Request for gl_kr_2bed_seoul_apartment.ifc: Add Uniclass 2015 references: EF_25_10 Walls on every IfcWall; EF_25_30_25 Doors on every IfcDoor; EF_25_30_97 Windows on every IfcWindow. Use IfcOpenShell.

First a look at what the model holds.

```python
import ifcopenshell

model = ifcopenshell.open("gl_kr_2bed_seoul_apartment.ifc")
print(model.schema)
print("classifications:", [c.Name for c in model.by_type("IfcClassification")])
for ifc_class in ("IfcDoor", "IfcRoof", "IfcStair", "IfcWall", "IfcWindow"):
    print(ifc_class, len(model.by_type(ifc_class)))
```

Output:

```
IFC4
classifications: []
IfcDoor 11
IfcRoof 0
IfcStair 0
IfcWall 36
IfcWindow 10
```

```python
import ifcopenshell
import ifcopenshell.api.classification

model = ifcopenshell.open("gl_kr_2bed_seoul_apartment.ifc")

system = ifcopenshell.api.classification.add_classification(model, classification="Uniclass 2015")

codes = {
    "IfcWall": ("EF_25_10", "Walls"),
    "IfcDoor": ("EF_25_30_25", "Doors"),
    "IfcWindow": ("EF_25_30_97", "Windows"),
}
for ifc_class, (code, name) in codes.items():
    products = model.by_type(ifc_class)
    ifcopenshell.api.classification.add_reference(
        model, products=products, classification=system, identification=code, name=name
    )
    print(code, len(products))

model.write("gl_kr_2bed_seoul_apartment-out.ifc")
```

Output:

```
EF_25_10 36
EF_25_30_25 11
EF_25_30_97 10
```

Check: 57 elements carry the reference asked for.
